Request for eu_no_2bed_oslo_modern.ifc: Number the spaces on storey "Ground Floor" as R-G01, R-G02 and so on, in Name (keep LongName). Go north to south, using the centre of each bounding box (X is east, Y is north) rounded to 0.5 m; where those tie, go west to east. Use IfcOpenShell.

First a look at what the model holds.

```python
import ifcopenshell
import ifcopenshell.util.element
import ifcopenshell.util.placement

model = ifcopenshell.open("eu_no_2bed_oslo_modern.ifc")
print(model.schema)
storey = next(s for s in model.by_type("IfcBuildingStorey") if s.Name == "Ground Floor")
spaces = [e for e in ifcopenshell.util.element.get_decomposition(storey) if e.is_a("IfcSpace")]
for e in sorted(spaces, key=lambda e: e.id()):
    origin = ifcopenshell.util.placement.get_local_placement(e.ObjectPlacement)[:3, 3]
    print(e.id(), e.Name, e.LongName, origin.round(2) + 0.0, sep=" | ")
```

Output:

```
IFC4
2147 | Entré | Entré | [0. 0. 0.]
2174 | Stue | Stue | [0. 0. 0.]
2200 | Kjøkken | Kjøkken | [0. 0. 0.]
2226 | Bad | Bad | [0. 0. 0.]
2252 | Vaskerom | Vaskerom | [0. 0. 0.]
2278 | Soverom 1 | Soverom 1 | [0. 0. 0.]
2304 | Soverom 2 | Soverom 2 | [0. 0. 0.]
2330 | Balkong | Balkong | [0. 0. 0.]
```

```python
import ifcopenshell
import ifcopenshell.geom
import ifcopenshell.util.element
import ifcopenshell.util.shape

model = ifcopenshell.open("eu_no_2bed_oslo_modern.ifc")
settings = ifcopenshell.geom.settings()
settings.set("use-world-coords", True)


def centre(element):
    shape = ifcopenshell.geom.create_shape(settings, element)
    return ifcopenshell.util.shape.get_bbox_centroid(shape.geometry)


storey = next(s for s in model.by_type("IfcBuildingStorey") if s.Name == "Ground Floor")
spaces = [e for e in ifcopenshell.util.element.get_decomposition(storey) if e.is_a("IfcSpace")]

# Insertion points can sit at a corner or the storey origin, so sort by the geometry (in metres).
centres = {e: centre(e) for e in spaces}
spaces.sort(key=lambda e: (-round(centres[e][1] / 0.5), centres[e][0]))

for i, e in enumerate(spaces, start=1):
    number = f"R-G{i:02d}"
    e.Name = number
    print(e.id(), number)

model.write("eu_no_2bed_oslo_modern_v2.ifc")
```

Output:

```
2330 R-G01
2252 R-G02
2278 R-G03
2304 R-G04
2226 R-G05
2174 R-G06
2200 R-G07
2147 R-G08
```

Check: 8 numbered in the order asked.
